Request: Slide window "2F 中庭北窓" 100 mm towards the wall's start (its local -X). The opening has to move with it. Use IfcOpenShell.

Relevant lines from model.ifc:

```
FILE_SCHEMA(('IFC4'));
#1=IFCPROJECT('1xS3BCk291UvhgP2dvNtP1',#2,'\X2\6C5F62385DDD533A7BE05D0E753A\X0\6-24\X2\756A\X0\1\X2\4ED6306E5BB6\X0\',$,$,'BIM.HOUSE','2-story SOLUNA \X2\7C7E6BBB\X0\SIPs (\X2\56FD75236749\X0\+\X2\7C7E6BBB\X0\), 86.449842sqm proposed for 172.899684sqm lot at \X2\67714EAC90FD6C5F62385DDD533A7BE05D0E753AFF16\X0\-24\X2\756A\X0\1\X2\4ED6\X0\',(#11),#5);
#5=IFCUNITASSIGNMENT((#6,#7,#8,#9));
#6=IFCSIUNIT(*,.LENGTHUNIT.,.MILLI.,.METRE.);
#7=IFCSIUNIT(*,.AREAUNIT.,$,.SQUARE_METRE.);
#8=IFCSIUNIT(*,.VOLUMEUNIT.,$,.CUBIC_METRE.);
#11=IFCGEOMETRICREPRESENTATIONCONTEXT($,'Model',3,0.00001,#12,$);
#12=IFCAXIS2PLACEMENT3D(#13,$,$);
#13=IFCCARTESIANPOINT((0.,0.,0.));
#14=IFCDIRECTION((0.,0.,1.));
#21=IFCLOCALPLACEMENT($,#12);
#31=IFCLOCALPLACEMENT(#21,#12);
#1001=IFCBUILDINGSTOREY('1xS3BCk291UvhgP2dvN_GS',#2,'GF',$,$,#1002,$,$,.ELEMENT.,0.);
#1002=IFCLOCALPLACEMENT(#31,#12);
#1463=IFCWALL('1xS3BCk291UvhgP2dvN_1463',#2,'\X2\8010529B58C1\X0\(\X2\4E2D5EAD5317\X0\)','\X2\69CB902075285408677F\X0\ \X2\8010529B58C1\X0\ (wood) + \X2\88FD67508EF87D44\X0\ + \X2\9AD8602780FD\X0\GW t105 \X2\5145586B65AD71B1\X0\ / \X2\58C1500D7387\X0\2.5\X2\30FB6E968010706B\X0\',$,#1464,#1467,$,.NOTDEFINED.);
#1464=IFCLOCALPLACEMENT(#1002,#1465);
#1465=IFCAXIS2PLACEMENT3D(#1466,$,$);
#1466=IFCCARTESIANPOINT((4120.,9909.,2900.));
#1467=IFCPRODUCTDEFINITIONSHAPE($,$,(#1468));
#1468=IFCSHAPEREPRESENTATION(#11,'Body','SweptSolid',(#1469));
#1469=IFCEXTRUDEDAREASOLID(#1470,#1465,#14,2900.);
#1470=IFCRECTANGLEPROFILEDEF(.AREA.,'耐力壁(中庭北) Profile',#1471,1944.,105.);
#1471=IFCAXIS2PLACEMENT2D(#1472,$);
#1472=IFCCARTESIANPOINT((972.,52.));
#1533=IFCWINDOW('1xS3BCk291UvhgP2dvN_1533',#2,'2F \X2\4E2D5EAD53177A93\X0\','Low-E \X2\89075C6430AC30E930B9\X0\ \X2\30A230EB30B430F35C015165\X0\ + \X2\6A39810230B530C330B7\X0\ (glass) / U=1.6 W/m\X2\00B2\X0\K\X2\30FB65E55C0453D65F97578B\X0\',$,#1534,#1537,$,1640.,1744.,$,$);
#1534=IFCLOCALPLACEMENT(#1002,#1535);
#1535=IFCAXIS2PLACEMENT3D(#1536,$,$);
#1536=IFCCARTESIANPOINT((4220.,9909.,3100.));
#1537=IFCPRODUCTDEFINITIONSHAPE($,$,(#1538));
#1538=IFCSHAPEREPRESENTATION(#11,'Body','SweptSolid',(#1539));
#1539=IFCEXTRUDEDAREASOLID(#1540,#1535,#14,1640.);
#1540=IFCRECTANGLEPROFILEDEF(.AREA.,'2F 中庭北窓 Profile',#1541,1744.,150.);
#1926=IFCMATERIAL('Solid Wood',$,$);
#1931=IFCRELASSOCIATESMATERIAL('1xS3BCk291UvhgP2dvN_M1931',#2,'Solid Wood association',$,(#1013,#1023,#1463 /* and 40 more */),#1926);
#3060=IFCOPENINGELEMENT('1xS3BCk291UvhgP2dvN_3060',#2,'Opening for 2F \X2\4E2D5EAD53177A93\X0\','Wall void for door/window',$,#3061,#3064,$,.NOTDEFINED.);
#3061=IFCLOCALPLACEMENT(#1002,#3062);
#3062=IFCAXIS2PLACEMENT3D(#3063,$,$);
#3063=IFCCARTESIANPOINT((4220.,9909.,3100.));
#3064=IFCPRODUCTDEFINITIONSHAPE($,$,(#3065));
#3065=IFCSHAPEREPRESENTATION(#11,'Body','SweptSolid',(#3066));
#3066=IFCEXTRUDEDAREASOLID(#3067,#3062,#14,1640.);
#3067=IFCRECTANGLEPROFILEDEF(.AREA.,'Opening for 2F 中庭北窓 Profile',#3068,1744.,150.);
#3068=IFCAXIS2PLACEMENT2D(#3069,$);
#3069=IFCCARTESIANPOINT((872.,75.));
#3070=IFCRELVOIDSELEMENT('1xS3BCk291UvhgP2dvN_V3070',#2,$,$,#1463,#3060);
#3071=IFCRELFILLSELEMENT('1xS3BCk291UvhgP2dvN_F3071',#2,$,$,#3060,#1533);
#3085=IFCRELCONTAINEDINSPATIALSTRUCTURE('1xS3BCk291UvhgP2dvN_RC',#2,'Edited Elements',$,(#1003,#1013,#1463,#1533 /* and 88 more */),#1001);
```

```python
import ifcopenshell
import ifcopenshell.api.geometry
import ifcopenshell.util.placement
import ifcopenshell.util.unit

model = ifcopenshell.open("model.ifc")
unit_scale = ifcopenshell.util.unit.calculate_unit_scale(model)

window = model.by_guid("1xS3BCk291UvhgP2dvN_1533")
opening = window.FillsVoids[0].RelatingOpeningElement
wall = opening.VoidsElements[0].RelatingBuildingElement

wall_matrix = ifcopenshell.util.placement.get_local_placement(wall.ObjectPlacement)
shift = wall_matrix[:3, 0] * -0.1 / unit_scale
before = ifcopenshell.util.placement.get_local_placement(window.ObjectPlacement)[:3, 3].copy()

# The window is not placed relative to its opening, so move both.
for product in (opening, window):
    matrix = ifcopenshell.util.placement.get_local_placement(product.ObjectPlacement)
    matrix[:3, 3] += shift
    ifcopenshell.api.geometry.edit_object_placement(model, product=product, matrix=matrix, is_si=False)

after = ifcopenshell.util.placement.get_local_placement(window.ObjectPlacement)[:3, 3]
print("window moved by", (after - before).round(3) + 0.0)

model.write("model_v2.ifc")
```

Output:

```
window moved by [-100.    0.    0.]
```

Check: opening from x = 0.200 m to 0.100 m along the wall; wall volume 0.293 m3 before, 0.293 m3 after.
